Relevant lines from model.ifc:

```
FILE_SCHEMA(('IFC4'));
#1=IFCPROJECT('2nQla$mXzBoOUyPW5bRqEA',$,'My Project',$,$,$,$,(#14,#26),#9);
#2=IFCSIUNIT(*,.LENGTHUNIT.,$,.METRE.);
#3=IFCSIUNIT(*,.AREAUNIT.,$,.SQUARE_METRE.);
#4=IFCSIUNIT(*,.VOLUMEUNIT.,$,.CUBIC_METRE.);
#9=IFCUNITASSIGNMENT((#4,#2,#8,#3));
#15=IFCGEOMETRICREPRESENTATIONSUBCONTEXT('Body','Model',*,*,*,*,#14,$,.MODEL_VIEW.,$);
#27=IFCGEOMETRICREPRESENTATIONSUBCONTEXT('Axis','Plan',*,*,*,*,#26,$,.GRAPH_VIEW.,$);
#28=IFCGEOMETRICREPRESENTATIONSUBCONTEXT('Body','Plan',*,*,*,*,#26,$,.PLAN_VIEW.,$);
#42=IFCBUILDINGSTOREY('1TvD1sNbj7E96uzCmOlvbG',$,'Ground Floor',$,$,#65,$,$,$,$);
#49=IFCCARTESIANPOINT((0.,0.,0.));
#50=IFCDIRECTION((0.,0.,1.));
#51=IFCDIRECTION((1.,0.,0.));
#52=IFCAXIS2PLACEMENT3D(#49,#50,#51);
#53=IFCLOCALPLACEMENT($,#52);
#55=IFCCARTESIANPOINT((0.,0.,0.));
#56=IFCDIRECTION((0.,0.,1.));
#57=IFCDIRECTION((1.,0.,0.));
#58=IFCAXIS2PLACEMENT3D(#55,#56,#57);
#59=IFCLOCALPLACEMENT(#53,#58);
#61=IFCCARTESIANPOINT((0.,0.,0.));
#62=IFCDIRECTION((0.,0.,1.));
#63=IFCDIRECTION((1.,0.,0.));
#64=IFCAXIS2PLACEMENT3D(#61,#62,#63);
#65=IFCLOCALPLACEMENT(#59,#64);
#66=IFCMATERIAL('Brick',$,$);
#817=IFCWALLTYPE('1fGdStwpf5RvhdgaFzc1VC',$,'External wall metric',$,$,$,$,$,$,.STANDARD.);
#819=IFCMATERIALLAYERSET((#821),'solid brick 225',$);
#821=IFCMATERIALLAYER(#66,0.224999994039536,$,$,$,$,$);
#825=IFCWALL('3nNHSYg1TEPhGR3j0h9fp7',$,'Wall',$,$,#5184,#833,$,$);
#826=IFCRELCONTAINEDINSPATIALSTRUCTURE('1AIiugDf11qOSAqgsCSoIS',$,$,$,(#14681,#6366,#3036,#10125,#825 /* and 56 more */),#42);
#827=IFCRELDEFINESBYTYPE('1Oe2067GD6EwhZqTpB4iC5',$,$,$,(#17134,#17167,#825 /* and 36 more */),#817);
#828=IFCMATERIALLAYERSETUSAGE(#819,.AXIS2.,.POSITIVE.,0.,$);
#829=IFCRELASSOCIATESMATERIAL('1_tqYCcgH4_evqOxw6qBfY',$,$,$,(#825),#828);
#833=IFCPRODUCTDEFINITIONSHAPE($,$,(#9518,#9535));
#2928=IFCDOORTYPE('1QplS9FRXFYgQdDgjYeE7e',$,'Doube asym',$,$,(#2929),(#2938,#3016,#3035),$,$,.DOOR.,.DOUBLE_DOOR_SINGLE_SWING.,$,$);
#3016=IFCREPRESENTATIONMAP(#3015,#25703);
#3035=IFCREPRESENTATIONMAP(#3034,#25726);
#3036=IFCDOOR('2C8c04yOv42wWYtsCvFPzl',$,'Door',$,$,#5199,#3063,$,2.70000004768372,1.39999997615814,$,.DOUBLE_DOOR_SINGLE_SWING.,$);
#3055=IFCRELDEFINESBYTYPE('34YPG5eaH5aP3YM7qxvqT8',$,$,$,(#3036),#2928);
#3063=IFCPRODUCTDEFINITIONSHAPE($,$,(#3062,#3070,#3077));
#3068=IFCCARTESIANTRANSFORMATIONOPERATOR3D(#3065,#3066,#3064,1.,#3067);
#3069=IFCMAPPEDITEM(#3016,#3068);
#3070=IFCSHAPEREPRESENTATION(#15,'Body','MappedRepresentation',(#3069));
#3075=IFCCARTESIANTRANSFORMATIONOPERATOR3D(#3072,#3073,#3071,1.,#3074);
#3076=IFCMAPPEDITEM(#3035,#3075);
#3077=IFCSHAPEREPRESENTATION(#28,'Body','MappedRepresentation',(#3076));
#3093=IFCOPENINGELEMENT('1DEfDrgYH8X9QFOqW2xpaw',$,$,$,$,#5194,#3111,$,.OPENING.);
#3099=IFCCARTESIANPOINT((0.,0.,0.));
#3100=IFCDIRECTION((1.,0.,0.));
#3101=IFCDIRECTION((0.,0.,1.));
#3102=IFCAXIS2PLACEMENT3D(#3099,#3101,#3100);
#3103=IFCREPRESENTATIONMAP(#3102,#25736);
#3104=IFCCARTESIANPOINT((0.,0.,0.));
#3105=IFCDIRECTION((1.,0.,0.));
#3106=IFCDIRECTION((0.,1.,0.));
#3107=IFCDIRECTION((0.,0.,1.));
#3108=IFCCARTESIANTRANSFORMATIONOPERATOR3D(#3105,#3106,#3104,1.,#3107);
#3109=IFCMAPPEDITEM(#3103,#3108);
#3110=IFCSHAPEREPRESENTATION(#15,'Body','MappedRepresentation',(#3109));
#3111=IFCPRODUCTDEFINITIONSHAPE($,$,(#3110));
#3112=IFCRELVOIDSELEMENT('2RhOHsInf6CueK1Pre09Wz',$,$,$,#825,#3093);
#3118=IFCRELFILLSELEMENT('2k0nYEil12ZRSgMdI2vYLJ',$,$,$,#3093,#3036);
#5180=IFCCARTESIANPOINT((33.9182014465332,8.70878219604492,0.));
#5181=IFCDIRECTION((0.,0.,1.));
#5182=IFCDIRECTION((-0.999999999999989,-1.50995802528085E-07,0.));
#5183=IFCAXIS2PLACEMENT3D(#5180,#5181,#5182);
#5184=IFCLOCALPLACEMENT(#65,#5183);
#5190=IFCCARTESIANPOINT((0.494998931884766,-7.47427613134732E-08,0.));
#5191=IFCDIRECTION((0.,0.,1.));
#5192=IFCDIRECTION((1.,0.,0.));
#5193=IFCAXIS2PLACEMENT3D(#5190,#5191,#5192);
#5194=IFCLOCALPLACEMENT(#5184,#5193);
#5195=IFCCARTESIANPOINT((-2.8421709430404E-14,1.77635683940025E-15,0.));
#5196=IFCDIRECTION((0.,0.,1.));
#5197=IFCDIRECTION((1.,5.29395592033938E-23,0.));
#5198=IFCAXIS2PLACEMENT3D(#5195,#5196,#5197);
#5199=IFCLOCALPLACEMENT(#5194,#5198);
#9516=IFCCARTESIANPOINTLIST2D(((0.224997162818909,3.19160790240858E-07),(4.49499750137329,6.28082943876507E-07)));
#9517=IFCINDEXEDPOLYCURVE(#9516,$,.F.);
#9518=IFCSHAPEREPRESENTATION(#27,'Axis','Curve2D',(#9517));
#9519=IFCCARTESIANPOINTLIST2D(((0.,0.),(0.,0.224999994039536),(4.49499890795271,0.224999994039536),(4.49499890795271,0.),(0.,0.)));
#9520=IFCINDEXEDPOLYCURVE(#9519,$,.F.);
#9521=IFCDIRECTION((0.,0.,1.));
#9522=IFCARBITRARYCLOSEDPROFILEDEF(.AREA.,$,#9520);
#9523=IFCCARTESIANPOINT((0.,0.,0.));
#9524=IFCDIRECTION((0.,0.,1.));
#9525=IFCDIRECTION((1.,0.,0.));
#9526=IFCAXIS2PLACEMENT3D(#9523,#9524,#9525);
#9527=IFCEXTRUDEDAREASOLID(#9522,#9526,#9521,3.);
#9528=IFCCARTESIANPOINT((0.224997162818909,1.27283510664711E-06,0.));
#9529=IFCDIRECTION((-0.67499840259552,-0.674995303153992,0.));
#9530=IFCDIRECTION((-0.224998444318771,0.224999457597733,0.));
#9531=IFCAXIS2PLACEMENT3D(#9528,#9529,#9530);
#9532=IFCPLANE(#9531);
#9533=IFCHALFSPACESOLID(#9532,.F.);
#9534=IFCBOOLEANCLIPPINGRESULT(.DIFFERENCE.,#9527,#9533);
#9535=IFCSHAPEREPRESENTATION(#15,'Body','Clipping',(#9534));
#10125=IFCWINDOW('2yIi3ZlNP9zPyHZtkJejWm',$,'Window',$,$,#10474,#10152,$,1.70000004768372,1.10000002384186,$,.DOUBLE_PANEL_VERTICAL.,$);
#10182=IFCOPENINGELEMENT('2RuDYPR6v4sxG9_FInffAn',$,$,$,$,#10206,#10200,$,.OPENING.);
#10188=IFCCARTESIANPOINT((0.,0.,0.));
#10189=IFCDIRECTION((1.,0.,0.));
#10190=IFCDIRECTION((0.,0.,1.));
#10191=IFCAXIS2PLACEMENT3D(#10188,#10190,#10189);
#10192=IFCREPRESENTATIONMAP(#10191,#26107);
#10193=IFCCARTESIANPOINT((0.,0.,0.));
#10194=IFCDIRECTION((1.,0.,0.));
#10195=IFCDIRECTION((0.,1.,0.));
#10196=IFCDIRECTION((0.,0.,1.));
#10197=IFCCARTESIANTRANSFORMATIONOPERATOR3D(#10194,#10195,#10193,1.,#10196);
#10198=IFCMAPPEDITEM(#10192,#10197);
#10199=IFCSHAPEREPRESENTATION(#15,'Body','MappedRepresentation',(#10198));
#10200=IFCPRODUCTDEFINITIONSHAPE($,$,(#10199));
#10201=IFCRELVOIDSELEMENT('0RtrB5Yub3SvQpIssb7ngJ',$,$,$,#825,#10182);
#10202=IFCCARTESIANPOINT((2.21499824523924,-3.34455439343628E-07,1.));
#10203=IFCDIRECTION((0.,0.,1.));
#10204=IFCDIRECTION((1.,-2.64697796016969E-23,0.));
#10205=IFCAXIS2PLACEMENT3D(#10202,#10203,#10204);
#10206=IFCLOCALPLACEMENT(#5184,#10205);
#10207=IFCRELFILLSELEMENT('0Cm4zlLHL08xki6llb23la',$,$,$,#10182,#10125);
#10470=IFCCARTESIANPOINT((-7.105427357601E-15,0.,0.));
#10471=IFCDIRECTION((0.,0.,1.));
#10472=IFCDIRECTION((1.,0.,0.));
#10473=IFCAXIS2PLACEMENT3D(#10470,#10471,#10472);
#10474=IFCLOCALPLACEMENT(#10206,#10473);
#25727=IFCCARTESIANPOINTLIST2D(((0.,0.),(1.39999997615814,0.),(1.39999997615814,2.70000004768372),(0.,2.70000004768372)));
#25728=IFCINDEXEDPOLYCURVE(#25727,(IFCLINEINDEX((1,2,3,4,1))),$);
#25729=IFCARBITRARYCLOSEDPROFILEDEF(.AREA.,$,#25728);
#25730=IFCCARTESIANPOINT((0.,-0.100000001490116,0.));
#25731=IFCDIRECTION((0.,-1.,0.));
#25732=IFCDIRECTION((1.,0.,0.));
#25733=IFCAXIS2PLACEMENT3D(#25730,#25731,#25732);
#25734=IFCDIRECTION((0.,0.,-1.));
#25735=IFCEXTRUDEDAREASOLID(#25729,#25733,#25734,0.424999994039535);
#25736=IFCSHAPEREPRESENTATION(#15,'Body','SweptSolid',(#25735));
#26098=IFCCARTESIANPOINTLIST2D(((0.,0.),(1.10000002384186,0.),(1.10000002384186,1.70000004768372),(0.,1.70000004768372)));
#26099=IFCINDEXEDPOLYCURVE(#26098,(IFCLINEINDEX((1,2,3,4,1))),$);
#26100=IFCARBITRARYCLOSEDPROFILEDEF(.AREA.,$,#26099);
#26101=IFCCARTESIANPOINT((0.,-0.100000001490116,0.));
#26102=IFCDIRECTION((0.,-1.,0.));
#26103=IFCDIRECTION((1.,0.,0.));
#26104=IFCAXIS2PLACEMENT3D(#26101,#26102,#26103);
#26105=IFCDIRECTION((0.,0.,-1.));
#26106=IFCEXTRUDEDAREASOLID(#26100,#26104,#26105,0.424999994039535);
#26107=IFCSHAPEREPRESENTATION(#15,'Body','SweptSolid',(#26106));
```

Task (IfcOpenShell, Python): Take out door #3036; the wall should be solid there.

```python
import ifcopenshell
import ifcopenshell.api.feature
import ifcopenshell.api.root
import ifcopenshell.geom
import ifcopenshell.util.shape

model = ifcopenshell.open("model.ifc")
settings = ifcopenshell.geom.settings()


def volume(element):
    """Net volume in cubic metres, openings subtracted."""
    shape = ifcopenshell.geom.create_shape(settings, element)
    return ifcopenshell.util.shape.get_volume(shape.geometry)


door = model.by_id(3036)
opening = door.FillsVoids[0].RelatingOpeningElement
wall = opening.VoidsElements[0].RelatingBuildingElement
before = volume(wall)

ifcopenshell.api.root.remove_product(model, product=door)
ifcopenshell.api.feature.remove_feature(model, feature=opening)

after = volume(wall)

print(f"wall volume {before:.3f} -> {after:.3f} m3")

model.write("model-out.ifc")
```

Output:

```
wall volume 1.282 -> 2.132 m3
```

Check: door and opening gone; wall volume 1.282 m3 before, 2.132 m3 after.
